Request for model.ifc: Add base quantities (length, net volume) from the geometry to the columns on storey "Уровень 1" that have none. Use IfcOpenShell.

First a look at what the model holds.

```python
import ifcopenshell
import ifcopenshell.util.element
import ifcopenshell.util.unit

model = ifcopenshell.open("model.ifc")
print(model.schema)
for unit_type in ("LENGTHUNIT", "AREAUNIT", "VOLUMEUNIT"):
    print(unit_type, ifcopenshell.util.unit.calculate_unit_scale(model, unit_type))
storey = next(s for s in model.by_type("IfcBuildingStorey") if s.Name == "Уровень 1")
columns = [e for e in ifcopenshell.util.element.get_decomposition(storey) if e.is_a("IfcColumn")]
for e in sorted(columns, key=lambda e: e.id()):
    print(e.id(), e.is_a(), e.Name, list(ifcopenshell.util.element.get_psets(e, qtos_only=True)), sep=" | ")
```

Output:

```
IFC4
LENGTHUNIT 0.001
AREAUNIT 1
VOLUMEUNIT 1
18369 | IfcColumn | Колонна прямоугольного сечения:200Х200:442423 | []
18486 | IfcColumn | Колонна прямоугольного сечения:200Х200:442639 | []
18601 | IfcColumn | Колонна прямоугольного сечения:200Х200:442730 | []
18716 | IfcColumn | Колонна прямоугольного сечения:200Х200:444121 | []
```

```python
import ifcopenshell
import ifcopenshell.api.pset
import ifcopenshell.geom
import ifcopenshell.util.element
import ifcopenshell.util.shape
import ifcopenshell.util.unit

model = ifcopenshell.open("model.ifc")
unit_scale = ifcopenshell.util.unit.calculate_unit_scale(model)
volume_scale = ifcopenshell.util.unit.calculate_unit_scale(model, "VOLUMEUNIT")
settings = ifcopenshell.geom.settings()

storey = next(s for s in model.by_type("IfcBuildingStorey") if s.Name == "Уровень 1")
columns = [e for e in ifcopenshell.util.element.get_decomposition(storey) if e.is_a("IfcColumn")]

for e in sorted(columns, key=lambda e: e.id()):
    if ifcopenshell.util.element.get_psets(e, qtos_only=True, should_inherit=False):
        continue
    # Geometry comes back in metres, in the element's own axes.
    shape = ifcopenshell.geom.create_shape(settings, e)
    values = {
        "Length": ifcopenshell.util.shape.get_z(shape.geometry) / unit_scale,
        "NetVolume": ifcopenshell.util.shape.get_volume(shape.geometry) / volume_scale,
    }
    qto = ifcopenshell.api.pset.add_qto(model, product=e, name="Qto_ColumnBaseQuantities")
    ifcopenshell.api.pset.edit_qto(model, qto=qto, properties=values)
    print(e.id(), {k: round(v, 3) for k, v in values.items()})

model.write("model_rev.ifc")
```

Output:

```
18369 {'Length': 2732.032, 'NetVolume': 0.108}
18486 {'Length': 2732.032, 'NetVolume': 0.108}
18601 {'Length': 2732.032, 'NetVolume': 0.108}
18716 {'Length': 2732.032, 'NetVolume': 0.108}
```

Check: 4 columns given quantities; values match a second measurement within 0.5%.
